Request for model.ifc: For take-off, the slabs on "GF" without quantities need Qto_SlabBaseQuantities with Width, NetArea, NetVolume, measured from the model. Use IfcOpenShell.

First a look at what the model holds.

```python
import ifcopenshell
import ifcopenshell.util.element
import ifcopenshell.util.unit

model = ifcopenshell.open("model.ifc")
print(model.schema)
for unit_type in ("LENGTHUNIT", "AREAUNIT", "VOLUMEUNIT"):
    print(unit_type, ifcopenshell.util.unit.calculate_unit_scale(model, unit_type))
storey = next(s for s in model.by_type("IfcBuildingStorey") if s.Name == "GF")
slabs = [e for e in ifcopenshell.util.element.get_decomposition(storey) if e.is_a("IfcSlab")]
for e in sorted(slabs, key=lambda e: e.id()):
    print(e.id(), e.is_a(), e.Name, list(ifcopenshell.util.element.get_psets(e, qtos_only=True)), sep=" | ")
```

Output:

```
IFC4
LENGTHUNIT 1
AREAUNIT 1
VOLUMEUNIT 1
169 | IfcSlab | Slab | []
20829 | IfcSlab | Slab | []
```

```python
import ifcopenshell
import ifcopenshell.api.pset
import ifcopenshell.geom
import ifcopenshell.util.element
import ifcopenshell.util.shape
import ifcopenshell.util.unit

model = ifcopenshell.open("model.ifc")
unit_scale = ifcopenshell.util.unit.calculate_unit_scale(model)
area_scale = ifcopenshell.util.unit.calculate_unit_scale(model, "AREAUNIT")
volume_scale = ifcopenshell.util.unit.calculate_unit_scale(model, "VOLUMEUNIT")
settings = ifcopenshell.geom.settings()

storey = next(s for s in model.by_type("IfcBuildingStorey") if s.Name == "GF")
slabs = [e for e in ifcopenshell.util.element.get_decomposition(storey) if e.is_a("IfcSlab")]

for e in sorted(slabs, key=lambda e: e.id()):
    if ifcopenshell.util.element.get_psets(e, qtos_only=True, should_inherit=False):
        continue
    # Geometry comes back in metres, in the element's own axes.
    shape = ifcopenshell.geom.create_shape(settings, e)
    values = {
        "Width": ifcopenshell.util.shape.get_z(shape.geometry) / unit_scale,
        "NetArea": ifcopenshell.util.shape.get_footprint_area(shape.geometry) / area_scale,
        "NetVolume": ifcopenshell.util.shape.get_volume(shape.geometry) / volume_scale,
    }
    qto = ifcopenshell.api.pset.add_qto(model, product=e, name="Qto_SlabBaseQuantities")
    ifcopenshell.api.pset.edit_qto(model, qto=qto, properties=values)
    print(e.id(), {k: round(v, 3) for k, v in values.items()})

model.write("model_updated.ifc")
```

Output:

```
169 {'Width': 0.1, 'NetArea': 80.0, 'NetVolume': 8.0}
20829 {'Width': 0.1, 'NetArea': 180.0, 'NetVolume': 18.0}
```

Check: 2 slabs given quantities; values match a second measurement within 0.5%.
